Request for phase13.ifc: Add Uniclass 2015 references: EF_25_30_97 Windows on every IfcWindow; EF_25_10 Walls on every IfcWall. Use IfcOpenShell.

First a look at what the model holds.

```python
import ifcopenshell

model = ifcopenshell.open("phase13.ifc")
print(model.schema)
print("classifications:", [c.Name for c in model.by_type("IfcClassification")])
for ifc_class in ("IfcDoor", "IfcRoof", "IfcStair", "IfcWall", "IfcWindow"):
    print(ifc_class, len(model.by_type(ifc_class)))
```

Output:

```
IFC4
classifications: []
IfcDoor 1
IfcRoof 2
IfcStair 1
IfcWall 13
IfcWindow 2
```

```python
import ifcopenshell
import ifcopenshell.api.classification

model = ifcopenshell.open("phase13.ifc")

system = ifcopenshell.api.classification.add_classification(model, classification="Uniclass 2015")

codes = {
    "IfcWindow": ("EF_25_30_97", "Windows"),
    "IfcWall": ("EF_25_10", "Walls"),
}
for ifc_class, (code, name) in codes.items():
    products = model.by_type(ifc_class)
    ifcopenshell.api.classification.add_reference(
        model, products=products, classification=system, identification=code, name=name
    )
    print(code, len(products))

model.write("phase13_edited.ifc")
```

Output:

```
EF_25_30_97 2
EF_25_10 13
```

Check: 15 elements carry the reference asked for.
